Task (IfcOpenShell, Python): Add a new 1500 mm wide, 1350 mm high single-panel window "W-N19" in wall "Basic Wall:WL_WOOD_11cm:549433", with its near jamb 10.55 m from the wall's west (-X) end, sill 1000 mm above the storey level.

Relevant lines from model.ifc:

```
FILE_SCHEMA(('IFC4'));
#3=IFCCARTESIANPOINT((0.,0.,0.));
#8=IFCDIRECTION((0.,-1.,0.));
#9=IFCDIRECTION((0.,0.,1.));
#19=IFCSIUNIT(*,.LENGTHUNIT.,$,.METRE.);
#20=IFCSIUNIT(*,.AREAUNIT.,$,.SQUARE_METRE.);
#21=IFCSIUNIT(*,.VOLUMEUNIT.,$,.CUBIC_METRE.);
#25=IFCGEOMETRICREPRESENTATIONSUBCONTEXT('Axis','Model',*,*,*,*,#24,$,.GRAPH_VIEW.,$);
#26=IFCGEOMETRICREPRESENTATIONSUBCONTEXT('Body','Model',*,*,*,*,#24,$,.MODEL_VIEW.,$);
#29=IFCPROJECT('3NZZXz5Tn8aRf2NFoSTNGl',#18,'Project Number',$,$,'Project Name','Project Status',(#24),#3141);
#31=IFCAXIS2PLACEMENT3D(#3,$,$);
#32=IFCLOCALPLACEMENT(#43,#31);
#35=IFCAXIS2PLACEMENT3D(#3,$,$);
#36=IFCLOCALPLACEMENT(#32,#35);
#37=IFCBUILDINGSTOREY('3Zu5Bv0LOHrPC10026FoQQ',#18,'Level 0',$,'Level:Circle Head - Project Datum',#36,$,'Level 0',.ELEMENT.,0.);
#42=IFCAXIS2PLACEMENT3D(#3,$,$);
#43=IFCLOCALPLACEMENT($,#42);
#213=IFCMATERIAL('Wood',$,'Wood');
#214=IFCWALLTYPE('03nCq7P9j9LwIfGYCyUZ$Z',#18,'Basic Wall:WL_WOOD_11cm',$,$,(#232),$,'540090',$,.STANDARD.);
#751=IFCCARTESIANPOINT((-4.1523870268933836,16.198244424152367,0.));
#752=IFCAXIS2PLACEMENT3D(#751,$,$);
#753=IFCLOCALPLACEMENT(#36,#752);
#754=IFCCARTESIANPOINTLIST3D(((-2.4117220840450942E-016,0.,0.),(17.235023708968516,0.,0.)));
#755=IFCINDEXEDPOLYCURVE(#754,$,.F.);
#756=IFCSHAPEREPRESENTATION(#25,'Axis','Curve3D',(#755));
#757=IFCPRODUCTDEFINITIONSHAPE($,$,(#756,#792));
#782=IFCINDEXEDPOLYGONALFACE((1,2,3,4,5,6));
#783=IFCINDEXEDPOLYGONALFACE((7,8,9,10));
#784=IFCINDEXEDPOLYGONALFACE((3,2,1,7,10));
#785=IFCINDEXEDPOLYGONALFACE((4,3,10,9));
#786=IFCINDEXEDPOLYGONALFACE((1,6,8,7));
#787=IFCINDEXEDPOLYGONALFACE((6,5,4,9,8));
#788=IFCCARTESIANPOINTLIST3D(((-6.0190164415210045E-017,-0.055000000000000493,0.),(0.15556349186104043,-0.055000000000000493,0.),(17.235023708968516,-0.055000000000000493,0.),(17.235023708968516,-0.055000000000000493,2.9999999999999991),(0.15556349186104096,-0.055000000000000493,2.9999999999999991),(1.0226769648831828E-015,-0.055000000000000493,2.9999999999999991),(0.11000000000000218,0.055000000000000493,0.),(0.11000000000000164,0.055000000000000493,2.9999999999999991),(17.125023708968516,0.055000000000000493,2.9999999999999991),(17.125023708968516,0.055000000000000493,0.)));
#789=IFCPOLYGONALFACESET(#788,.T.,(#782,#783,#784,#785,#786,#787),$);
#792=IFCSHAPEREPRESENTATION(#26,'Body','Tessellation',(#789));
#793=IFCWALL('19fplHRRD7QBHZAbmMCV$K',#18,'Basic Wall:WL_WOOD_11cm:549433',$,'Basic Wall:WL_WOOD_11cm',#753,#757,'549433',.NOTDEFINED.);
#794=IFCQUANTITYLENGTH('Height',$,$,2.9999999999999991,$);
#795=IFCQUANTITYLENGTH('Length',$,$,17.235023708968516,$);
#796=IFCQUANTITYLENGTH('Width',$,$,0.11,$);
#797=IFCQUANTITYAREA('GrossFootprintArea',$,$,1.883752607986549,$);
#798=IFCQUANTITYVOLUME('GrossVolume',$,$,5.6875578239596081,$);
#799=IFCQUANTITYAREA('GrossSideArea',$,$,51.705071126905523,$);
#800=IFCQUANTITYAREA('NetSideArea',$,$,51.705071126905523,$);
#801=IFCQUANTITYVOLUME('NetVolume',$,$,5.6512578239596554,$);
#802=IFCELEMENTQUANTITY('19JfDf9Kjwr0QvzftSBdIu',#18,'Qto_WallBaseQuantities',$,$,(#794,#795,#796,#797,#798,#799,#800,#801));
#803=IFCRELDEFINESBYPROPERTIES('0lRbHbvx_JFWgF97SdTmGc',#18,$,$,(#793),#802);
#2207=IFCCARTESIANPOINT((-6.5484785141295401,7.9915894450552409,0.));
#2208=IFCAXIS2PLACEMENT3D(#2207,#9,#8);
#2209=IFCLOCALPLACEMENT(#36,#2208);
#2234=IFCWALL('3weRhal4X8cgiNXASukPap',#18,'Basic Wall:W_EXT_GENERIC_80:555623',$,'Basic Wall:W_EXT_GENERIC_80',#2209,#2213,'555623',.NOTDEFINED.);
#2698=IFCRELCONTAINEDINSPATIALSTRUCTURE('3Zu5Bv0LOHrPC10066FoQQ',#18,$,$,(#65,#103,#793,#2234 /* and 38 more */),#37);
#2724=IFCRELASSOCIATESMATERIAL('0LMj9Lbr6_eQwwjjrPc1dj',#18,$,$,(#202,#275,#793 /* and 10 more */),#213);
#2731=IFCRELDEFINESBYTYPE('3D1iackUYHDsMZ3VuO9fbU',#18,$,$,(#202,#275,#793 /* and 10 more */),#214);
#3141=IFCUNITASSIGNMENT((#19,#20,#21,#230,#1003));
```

```python
import numpy as np
import ifcopenshell
import ifcopenshell.api.feature
import ifcopenshell.api.geometry
import ifcopenshell.api.pset
import ifcopenshell.api.root
import ifcopenshell.api.spatial
import ifcopenshell.geom
import ifcopenshell.util.element
import ifcopenshell.util.placement
import ifcopenshell.util.representation
import ifcopenshell.util.shape
import ifcopenshell.util.unit

model = ifcopenshell.open("model.ifc")
unit_scale = ifcopenshell.util.unit.calculate_unit_scale(model)
area_scale = ifcopenshell.util.unit.calculate_unit_scale(model, "AREAUNIT")
volume_scale = ifcopenshell.util.unit.calculate_unit_scale(model, "VOLUMEUNIT")
settings = ifcopenshell.geom.settings()


def volume(element):
    """Net volume in cubic metres, openings subtracted."""
    shape = ifcopenshell.geom.create_shape(settings, element)
    return ifcopenshell.util.shape.get_volume(shape.geometry)


wall = model.by_guid("19fplHRRD7QBHZAbmMCV$K")
storey = ifcopenshell.util.element.get_container(wall, ifc_class="IfcBuildingStorey")
context = ifcopenshell.util.representation.get_context(model, "Model", "Body", "MODEL_VIEW")
before = volume(wall)

width, height, from_end, sill = 1.5, 1.35, 10.55, 1  # metres

# The wall runs along its own X axis, and the end named is its -X end.
wall_shape = ifcopenshell.geom.create_shape(settings, wall)
x, y, z = ifcopenshell.util.shape.get_vertices(wall_shape.geometry).T
start = x.min() + from_end
face, thickness = float(y.min()), float(y.max() - y.min())
wall_matrix = ifcopenshell.util.placement.get_local_placement(wall.ObjectPlacement)
level = ifcopenshell.util.placement.get_local_placement(storey.ObjectPlacement)[2, 3]


def in_wall(x, y):
    """Placement at x, y metres in the wall's axes, at sill height."""
    matrix = wall_matrix.copy()
    matrix[:, 3] = wall_matrix @ np.array([x / unit_scale, y / unit_scale, 0.0, 1.0])
    matrix[2, 3] = level + sill / unit_scale
    return matrix


# Opening: a box that overshoots both wall faces by 50 mm.
opening = ifcopenshell.api.root.create_entity(model, ifc_class="IfcOpeningElement", predefined_type="OPENING")
box = ifcopenshell.api.geometry.add_wall_representation(
    model, context=context, length=width, height=height, thickness=thickness + 0.1
)
ifcopenshell.api.geometry.assign_representation(model, product=opening, representation=box)
ifcopenshell.api.geometry.edit_object_placement(model, product=opening, matrix=in_wall(start, face - 0.05), is_si=False)
ifcopenshell.api.feature.add_feature(model, feature=opening, element=wall)

window = ifcopenshell.api.root.create_entity(model, ifc_class="IfcWindow", name="W-N19", predefined_type="WINDOW")
window.OverallWidth, window.OverallHeight = width / unit_scale, height / unit_scale
window.PartitioningType = "SINGLE_PANEL"
body = ifcopenshell.api.geometry.add_window_representation(
    model,
    context=context,
    overall_width=window.OverallWidth,
    overall_height=window.OverallHeight,
    partition_type="SINGLE_PANEL",
)
ifcopenshell.api.geometry.assign_representation(model, product=window, representation=body)
ifcopenshell.api.spatial.assign_container(model, products=[window], relating_structure=storey)
ifcopenshell.api.feature.add_filling(model, opening=opening, element=window)

# Centre the window in the wall's thickness.
ifcopenshell.api.geometry.edit_object_placement(model, product=window, matrix=in_wall(start, face), is_si=False)
window_shape = ifcopenshell.geom.create_shape(settings, window)
depth = ifcopenshell.util.shape.get_vertices(window_shape.geometry)[:, 1]
offset = face + thickness / 2 - (depth.min() + depth.max()) / 2
ifcopenshell.api.geometry.edit_object_placement(model, product=window, matrix=in_wall(start, offset), is_si=False)

after = volume(wall)

# Update the wall's stored quantities.
qto = model.by_id(ifcopenshell.util.element.get_pset(wall, "Qto_WallBaseQuantities", should_inherit=False)["id"])
ifcopenshell.api.pset.edit_qto(model, qto=qto, properties={
    "NetSideArea": after / thickness / area_scale,
    "NetVolume": after / volume_scale,
})

print(f"wall volume {before:.3f} -> {after:.3f} m3")

model.write("model_edited.ifc")
```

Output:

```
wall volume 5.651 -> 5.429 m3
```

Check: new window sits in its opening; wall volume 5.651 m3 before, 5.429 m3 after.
